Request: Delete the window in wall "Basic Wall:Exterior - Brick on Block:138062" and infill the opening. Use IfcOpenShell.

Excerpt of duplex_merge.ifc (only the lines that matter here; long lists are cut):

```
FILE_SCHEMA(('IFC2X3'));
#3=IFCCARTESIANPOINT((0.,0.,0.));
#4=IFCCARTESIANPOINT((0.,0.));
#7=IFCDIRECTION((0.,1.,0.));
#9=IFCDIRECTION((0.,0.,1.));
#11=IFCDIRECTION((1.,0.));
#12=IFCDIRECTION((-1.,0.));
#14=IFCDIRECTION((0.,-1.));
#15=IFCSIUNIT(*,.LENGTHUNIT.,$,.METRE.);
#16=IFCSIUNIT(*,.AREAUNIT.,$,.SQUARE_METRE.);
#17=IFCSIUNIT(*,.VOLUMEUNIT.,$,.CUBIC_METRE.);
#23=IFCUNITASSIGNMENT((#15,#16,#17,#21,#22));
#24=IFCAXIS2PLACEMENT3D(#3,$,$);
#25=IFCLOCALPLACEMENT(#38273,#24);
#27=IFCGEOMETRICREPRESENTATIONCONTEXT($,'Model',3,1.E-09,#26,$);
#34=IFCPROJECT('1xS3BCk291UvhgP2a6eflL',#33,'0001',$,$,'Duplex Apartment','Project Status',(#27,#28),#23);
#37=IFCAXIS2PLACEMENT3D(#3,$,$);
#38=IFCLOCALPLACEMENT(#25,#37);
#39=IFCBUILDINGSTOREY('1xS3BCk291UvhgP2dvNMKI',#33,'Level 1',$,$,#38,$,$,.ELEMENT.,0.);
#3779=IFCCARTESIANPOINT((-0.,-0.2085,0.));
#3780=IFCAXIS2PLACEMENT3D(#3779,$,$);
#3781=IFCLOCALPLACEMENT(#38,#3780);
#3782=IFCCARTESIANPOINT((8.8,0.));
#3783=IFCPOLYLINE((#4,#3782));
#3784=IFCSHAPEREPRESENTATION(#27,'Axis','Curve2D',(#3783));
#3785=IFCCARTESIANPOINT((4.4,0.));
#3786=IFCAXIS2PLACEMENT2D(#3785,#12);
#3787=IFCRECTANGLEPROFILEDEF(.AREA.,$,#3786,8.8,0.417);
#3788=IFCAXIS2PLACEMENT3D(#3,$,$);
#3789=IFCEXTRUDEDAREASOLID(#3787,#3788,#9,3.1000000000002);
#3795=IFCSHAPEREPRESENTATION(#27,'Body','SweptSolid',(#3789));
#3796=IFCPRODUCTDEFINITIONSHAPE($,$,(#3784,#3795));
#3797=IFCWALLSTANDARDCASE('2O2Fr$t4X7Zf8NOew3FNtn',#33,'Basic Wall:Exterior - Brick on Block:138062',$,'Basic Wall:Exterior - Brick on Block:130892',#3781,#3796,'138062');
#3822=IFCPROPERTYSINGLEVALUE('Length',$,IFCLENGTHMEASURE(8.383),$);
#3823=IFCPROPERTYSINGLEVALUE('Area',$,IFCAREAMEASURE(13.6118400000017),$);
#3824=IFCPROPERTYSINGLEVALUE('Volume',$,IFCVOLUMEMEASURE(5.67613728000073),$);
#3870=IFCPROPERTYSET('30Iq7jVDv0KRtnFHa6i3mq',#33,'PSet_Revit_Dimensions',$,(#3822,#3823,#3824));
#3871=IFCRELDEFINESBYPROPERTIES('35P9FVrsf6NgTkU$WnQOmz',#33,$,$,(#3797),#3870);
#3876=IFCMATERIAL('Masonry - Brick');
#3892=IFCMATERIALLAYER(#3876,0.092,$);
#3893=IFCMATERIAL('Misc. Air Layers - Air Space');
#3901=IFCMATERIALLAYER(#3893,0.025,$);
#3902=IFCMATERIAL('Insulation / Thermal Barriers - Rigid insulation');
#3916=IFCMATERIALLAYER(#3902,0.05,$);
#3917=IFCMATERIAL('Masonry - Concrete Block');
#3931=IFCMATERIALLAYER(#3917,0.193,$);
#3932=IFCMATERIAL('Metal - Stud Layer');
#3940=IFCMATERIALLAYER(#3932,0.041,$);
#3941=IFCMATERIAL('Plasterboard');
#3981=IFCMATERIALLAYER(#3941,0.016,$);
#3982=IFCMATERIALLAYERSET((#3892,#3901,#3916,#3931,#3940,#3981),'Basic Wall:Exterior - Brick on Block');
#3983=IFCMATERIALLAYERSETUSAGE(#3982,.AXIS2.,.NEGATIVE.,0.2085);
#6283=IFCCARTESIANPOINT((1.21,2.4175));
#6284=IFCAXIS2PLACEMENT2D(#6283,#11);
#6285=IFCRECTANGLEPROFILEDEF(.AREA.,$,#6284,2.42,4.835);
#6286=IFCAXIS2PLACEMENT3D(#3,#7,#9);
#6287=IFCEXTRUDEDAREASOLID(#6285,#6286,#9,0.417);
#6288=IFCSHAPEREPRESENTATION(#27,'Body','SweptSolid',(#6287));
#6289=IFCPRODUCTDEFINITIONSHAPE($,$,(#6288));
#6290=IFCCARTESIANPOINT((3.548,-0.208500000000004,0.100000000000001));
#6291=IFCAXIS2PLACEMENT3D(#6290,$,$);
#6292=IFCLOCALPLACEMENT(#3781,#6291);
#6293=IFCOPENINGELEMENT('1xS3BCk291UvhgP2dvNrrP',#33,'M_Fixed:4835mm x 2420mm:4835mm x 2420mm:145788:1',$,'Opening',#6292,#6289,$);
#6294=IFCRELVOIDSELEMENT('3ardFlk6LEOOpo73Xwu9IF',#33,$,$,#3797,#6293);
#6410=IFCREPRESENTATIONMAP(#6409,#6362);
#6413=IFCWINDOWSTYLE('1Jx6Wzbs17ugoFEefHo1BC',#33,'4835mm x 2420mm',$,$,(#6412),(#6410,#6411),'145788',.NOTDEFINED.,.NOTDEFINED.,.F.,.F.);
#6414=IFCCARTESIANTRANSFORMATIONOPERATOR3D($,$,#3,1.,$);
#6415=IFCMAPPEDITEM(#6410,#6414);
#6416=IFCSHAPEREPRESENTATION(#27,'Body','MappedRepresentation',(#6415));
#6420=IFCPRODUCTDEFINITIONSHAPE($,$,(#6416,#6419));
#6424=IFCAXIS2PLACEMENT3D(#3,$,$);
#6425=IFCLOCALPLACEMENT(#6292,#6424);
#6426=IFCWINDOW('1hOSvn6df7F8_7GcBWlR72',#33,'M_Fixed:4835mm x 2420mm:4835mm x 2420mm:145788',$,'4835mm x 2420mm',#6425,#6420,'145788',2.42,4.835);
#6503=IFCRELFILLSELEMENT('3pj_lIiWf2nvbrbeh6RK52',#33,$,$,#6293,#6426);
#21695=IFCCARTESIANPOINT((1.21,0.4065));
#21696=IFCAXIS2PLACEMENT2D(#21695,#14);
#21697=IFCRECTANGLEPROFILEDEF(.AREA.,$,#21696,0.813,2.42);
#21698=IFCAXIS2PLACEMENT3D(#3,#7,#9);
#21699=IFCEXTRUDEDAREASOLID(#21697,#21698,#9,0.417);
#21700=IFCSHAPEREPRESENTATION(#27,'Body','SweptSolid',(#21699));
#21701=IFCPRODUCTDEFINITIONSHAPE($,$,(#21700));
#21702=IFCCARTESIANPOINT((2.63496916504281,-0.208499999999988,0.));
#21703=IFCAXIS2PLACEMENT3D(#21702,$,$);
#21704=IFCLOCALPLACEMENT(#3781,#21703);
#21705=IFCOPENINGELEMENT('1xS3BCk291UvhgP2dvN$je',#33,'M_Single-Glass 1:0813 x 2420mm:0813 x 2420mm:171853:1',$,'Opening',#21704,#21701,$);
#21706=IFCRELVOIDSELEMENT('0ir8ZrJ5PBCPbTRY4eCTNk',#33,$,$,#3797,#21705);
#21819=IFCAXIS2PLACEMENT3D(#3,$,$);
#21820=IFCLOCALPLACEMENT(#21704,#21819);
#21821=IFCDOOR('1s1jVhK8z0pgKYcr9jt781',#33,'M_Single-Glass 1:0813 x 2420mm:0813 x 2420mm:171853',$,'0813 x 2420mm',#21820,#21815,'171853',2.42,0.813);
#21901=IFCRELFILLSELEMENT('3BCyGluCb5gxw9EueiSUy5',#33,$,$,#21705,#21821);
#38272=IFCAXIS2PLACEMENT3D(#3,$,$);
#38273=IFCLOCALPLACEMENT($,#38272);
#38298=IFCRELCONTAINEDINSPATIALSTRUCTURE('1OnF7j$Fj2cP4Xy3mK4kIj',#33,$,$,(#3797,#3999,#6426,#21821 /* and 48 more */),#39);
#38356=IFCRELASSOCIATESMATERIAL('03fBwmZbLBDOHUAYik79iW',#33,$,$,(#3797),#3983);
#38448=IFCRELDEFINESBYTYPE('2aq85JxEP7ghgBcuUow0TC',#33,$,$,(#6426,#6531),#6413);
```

```python
import ifcopenshell
import ifcopenshell.api.feature
import ifcopenshell.api.pset
import ifcopenshell.api.root
import ifcopenshell.geom
import ifcopenshell.util.element
import ifcopenshell.util.shape
import ifcopenshell.util.unit

model = ifcopenshell.open("duplex_merge.ifc")
area_scale = ifcopenshell.util.unit.calculate_unit_scale(model, "AREAUNIT")
volume_scale = ifcopenshell.util.unit.calculate_unit_scale(model, "VOLUMEUNIT")
settings = ifcopenshell.geom.settings()


def volume(element):
    """Net volume in cubic metres, openings subtracted."""
    shape = ifcopenshell.geom.create_shape(settings, element)
    return ifcopenshell.util.shape.get_volume(shape.geometry)


window = model.by_id(6426)
opening = window.FillsVoids[0].RelatingOpeningElement
wall = opening.VoidsElements[0].RelatingBuildingElement
before = volume(wall)

ifcopenshell.api.root.remove_product(model, product=window)
ifcopenshell.api.feature.remove_feature(model, feature=opening)

after = volume(wall)
thickness = 0.417  # wall thickness in metres

# Update the wall's stored quantities.
pset = model.by_id(ifcopenshell.util.element.get_pset(wall, "PSet_Revit_Dimensions", should_inherit=False)["id"])
ifcopenshell.api.pset.edit_pset(model, pset=pset, properties={
    "Area": model.create_entity("IfcAreaMeasure", after / thickness / area_scale),
    "Volume": model.create_entity("IfcVolumeMeasure", after / volume_scale),
})

print(f"wall volume {before:.3f} -> {after:.3f} m3")

model.write("duplex_merge_rev.ifc")
```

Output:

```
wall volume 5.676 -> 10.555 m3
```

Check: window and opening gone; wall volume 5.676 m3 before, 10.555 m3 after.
